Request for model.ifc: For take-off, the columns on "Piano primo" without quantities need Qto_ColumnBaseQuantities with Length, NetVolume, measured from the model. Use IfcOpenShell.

First a look at what the model holds.

```python
import ifcopenshell
import ifcopenshell.util.element
import ifcopenshell.util.unit

model = ifcopenshell.open("model.ifc")
print(model.schema)
for unit_type in ("LENGTHUNIT", "AREAUNIT", "VOLUMEUNIT"):
    print(unit_type, ifcopenshell.util.unit.calculate_unit_scale(model, unit_type))
storey = next(s for s in model.by_type("IfcBuildingStorey") if s.Name == "Piano primo")
columns = [e for e in ifcopenshell.util.element.get_decomposition(storey) if e.is_a("IfcColumn")]
for e in sorted(columns, key=lambda e: e.id()):
    print(e.id(), e.is_a(), e.Name, list(ifcopenshell.util.element.get_psets(e, qtos_only=True)), sep=" | ")
```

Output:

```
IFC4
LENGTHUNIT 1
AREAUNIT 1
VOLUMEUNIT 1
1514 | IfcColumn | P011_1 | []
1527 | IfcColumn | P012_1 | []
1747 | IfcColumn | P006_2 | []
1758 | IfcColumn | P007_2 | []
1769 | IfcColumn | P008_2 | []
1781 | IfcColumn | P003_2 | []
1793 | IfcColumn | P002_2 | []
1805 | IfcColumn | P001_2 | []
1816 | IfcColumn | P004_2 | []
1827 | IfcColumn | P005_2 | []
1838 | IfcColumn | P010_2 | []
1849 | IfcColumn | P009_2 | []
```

```python
import ifcopenshell
import ifcopenshell.api.pset
import ifcopenshell.geom
import ifcopenshell.util.element
import ifcopenshell.util.shape
import ifcopenshell.util.unit

model = ifcopenshell.open("model.ifc")
unit_scale = ifcopenshell.util.unit.calculate_unit_scale(model)
volume_scale = ifcopenshell.util.unit.calculate_unit_scale(model, "VOLUMEUNIT")
settings = ifcopenshell.geom.settings()

storey = next(s for s in model.by_type("IfcBuildingStorey") if s.Name == "Piano primo")
columns = [e for e in ifcopenshell.util.element.get_decomposition(storey) if e.is_a("IfcColumn")]

for e in sorted(columns, key=lambda e: e.id()):
    if ifcopenshell.util.element.get_psets(e, qtos_only=True, should_inherit=False):
        continue
    # Geometry comes back in metres, in the element's own axes.
    shape = ifcopenshell.geom.create_shape(settings, e)
    values = {
        "Length": ifcopenshell.util.shape.get_z(shape.geometry) / unit_scale,
        "NetVolume": ifcopenshell.util.shape.get_volume(shape.geometry) / volume_scale,
    }
    qto = ifcopenshell.api.pset.add_qto(model, product=e, name="Qto_ColumnBaseQuantities")
    ifcopenshell.api.pset.edit_qto(model, qto=qto, properties=values)
    print(e.id(), {k: round(v, 3) for k, v in values.items()})

model.write("model_updated.ifc")
```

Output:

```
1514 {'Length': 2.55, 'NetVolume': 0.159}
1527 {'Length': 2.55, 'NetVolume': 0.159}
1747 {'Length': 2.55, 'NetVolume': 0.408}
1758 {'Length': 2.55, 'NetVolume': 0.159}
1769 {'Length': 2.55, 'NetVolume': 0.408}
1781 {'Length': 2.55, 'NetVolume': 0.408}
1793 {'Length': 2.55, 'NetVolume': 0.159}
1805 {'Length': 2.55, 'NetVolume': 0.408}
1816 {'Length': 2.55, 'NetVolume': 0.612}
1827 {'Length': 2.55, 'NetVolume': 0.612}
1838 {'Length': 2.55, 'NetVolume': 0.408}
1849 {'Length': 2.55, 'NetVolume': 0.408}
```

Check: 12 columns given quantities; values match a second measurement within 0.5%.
